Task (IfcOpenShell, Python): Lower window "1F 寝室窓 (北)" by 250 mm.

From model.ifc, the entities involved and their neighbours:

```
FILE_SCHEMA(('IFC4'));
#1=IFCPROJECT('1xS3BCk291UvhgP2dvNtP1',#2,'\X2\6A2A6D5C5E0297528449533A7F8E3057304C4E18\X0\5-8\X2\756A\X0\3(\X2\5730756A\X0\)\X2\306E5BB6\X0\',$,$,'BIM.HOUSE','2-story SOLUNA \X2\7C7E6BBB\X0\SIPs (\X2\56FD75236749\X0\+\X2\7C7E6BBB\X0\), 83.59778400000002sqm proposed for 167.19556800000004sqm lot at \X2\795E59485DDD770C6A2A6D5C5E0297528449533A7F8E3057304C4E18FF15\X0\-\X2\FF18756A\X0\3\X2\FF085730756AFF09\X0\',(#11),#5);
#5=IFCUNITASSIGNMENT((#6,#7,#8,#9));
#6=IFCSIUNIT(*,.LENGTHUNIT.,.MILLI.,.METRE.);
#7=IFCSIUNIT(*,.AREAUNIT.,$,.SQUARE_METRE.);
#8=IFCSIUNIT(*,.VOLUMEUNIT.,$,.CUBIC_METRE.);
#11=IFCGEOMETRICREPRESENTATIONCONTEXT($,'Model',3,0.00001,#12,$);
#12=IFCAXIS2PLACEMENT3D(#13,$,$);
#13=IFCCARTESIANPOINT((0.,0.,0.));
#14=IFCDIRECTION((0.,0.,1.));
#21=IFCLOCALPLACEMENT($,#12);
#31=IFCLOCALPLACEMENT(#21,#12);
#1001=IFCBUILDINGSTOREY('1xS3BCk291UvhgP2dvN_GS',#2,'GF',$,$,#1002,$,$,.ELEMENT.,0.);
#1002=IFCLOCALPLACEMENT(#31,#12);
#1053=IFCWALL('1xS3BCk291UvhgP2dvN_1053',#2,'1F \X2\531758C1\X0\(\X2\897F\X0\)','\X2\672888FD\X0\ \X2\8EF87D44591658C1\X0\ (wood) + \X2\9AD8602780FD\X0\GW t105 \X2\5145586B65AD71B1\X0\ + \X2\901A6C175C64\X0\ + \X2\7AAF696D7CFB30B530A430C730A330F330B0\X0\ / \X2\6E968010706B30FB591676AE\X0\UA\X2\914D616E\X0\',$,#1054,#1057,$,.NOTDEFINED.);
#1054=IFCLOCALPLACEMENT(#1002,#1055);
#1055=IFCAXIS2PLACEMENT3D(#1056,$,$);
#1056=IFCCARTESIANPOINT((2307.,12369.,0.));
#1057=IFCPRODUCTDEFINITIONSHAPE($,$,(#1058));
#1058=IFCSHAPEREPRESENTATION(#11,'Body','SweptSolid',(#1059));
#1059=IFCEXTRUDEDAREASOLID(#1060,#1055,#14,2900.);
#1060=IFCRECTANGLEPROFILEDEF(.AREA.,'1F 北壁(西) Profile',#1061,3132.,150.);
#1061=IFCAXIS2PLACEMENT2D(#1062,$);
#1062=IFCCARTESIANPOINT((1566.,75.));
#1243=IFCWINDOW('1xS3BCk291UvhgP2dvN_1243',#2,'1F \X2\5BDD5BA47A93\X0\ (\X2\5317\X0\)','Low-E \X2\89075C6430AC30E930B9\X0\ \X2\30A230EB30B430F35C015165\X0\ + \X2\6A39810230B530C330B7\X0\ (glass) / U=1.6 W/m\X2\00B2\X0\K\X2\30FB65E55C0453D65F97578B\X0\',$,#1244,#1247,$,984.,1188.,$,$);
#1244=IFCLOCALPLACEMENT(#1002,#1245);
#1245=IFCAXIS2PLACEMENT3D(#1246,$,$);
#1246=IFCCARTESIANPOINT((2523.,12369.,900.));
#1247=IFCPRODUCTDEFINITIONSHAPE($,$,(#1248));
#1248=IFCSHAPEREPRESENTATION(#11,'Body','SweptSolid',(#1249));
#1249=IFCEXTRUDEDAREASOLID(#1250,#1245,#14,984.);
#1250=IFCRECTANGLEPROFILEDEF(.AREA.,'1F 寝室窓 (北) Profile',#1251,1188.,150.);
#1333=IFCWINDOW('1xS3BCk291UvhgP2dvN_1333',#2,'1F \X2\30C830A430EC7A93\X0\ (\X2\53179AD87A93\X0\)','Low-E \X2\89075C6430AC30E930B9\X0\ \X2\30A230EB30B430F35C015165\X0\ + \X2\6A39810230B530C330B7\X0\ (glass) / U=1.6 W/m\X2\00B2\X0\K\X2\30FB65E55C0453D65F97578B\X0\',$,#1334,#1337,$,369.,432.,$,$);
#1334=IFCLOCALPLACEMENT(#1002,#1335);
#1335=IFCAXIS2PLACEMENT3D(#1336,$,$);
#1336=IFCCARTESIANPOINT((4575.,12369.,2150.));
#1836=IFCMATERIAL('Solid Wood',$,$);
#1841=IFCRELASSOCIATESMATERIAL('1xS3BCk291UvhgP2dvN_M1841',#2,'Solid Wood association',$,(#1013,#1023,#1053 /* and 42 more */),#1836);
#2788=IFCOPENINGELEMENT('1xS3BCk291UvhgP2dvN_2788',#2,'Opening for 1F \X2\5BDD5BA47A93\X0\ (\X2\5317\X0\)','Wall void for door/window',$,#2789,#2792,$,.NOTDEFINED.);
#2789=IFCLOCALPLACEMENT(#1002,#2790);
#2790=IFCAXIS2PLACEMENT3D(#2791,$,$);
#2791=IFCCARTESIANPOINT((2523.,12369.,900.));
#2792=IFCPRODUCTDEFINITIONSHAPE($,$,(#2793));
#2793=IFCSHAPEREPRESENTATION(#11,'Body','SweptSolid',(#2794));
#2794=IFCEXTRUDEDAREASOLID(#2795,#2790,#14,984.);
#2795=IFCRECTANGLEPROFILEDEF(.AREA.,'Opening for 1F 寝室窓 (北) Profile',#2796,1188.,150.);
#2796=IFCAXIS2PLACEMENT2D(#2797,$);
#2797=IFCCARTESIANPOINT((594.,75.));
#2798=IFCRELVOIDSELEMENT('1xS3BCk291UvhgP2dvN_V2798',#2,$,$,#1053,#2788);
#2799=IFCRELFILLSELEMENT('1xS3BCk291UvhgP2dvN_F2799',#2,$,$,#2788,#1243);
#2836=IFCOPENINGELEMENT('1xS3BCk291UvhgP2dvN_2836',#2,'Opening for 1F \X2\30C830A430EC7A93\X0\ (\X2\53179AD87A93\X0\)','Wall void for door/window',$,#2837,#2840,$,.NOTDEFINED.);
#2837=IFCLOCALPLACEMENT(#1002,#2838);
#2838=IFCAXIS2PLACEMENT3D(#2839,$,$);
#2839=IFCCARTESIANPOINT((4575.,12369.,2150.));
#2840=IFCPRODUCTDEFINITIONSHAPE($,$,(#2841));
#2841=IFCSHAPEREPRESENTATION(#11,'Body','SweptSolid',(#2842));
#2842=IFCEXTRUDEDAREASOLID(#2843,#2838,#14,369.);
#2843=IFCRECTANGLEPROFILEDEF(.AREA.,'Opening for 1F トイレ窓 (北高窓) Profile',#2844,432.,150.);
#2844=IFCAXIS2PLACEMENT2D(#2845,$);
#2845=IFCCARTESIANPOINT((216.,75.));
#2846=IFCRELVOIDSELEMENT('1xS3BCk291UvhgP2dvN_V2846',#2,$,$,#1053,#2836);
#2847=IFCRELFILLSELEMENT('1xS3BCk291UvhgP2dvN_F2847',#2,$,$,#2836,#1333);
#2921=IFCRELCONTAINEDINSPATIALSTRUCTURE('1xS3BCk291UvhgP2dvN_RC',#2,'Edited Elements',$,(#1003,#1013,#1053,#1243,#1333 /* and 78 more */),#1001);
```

```python
import numpy as np
import ifcopenshell
import ifcopenshell.api.geometry
import ifcopenshell.util.placement
import ifcopenshell.util.unit

model = ifcopenshell.open("model.ifc")
unit_scale = ifcopenshell.util.unit.calculate_unit_scale(model)

window = model.by_id(1243)
opening = window.FillsVoids[0].RelatingOpeningElement
dz = -0.25 / unit_scale

shift = np.array([0.0, 0.0, dz])
# The window is not placed relative to its opening, so move both.
for product in (opening, window):
    matrix = ifcopenshell.util.placement.get_local_placement(product.ObjectPlacement)
    matrix[:3, 3] += shift
    ifcopenshell.api.geometry.edit_object_placement(model, product=product, matrix=matrix, is_si=False)

print(f"moved by {dz * unit_scale:+.3f} m")

model.write("model_v2.ifc")
```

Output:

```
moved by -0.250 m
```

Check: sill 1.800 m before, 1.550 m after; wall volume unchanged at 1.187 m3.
